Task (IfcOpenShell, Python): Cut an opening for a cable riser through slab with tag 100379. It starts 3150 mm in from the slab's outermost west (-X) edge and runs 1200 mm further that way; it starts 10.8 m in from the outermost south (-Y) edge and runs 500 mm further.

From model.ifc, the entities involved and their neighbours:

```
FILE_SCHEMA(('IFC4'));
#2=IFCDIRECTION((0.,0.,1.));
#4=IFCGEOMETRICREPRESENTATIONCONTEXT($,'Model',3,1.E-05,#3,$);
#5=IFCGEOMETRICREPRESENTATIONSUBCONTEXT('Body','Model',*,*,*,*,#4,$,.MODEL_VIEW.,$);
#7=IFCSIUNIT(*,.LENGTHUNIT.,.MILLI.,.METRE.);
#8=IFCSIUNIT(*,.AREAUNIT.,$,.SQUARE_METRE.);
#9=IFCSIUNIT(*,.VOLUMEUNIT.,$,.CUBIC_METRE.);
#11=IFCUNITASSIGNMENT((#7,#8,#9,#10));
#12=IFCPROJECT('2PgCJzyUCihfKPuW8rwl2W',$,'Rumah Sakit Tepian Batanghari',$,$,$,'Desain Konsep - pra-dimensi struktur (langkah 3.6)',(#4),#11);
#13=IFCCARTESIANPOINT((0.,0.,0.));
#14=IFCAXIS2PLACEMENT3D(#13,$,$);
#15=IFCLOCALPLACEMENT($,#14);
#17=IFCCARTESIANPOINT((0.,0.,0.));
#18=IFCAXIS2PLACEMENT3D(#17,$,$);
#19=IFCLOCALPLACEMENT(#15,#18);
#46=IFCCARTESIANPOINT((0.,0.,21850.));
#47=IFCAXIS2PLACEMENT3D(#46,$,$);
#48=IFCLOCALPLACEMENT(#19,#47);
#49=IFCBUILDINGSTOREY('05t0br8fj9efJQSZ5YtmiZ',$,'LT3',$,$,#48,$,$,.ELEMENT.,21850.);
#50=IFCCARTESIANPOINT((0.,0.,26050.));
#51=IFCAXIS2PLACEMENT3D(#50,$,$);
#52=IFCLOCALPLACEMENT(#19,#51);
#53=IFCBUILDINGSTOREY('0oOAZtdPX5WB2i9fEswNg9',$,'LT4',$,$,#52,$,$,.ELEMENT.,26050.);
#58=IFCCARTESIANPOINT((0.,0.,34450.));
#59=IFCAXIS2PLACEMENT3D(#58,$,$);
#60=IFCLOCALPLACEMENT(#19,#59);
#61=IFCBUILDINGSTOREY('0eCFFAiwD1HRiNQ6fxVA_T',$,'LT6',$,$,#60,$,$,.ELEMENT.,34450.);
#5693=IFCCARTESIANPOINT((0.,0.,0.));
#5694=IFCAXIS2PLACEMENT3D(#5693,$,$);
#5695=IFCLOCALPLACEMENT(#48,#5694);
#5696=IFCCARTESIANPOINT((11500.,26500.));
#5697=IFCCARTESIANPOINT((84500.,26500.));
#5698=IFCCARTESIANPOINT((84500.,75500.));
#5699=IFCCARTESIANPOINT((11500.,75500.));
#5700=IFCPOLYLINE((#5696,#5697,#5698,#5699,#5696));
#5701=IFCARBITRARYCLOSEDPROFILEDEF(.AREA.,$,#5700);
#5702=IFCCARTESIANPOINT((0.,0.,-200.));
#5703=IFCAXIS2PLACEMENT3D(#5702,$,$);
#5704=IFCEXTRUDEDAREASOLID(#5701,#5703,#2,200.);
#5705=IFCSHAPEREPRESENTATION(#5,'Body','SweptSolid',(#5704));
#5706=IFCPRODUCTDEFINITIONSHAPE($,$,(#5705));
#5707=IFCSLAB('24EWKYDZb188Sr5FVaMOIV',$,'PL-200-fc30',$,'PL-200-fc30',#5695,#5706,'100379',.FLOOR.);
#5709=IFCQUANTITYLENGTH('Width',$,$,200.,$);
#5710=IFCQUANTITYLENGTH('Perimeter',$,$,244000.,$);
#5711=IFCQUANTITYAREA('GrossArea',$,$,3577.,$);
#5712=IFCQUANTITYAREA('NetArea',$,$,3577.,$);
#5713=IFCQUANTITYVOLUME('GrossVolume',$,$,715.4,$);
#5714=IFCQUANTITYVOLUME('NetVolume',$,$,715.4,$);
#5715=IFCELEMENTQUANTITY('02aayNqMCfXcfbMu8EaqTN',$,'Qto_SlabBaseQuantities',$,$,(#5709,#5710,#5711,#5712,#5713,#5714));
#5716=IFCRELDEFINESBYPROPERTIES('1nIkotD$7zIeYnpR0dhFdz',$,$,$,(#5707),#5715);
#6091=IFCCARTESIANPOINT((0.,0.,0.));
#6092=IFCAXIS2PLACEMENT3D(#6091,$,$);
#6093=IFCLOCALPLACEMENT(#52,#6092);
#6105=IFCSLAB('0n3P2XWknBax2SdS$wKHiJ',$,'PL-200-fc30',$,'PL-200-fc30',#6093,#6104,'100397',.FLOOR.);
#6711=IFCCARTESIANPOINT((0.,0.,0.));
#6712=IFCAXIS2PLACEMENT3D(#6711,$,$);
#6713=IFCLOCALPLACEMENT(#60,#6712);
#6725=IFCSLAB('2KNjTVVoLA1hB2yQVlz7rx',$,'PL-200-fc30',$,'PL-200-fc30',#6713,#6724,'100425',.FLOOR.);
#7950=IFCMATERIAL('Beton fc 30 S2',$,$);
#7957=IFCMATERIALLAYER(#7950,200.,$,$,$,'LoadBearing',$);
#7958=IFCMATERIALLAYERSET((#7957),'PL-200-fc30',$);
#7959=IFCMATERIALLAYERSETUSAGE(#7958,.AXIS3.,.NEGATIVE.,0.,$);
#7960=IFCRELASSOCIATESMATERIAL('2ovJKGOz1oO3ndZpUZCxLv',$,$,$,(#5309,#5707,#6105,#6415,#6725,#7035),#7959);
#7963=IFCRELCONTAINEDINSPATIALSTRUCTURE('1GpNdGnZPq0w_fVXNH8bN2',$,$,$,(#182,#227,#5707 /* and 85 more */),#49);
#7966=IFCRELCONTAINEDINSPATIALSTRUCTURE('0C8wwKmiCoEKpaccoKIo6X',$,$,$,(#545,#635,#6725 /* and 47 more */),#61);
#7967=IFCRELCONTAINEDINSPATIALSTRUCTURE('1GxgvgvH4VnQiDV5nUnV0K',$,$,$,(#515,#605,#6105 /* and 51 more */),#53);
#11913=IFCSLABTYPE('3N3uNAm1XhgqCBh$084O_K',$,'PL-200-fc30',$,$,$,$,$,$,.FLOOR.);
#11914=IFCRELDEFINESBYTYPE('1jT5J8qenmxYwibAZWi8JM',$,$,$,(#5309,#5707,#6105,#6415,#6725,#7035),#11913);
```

```python
import numpy as np
import ifcopenshell
import ifcopenshell.api.feature
import ifcopenshell.api.geometry
import ifcopenshell.api.pset
import ifcopenshell.api.root
import ifcopenshell.geom
import ifcopenshell.util.element
import ifcopenshell.util.placement
import ifcopenshell.util.representation
import ifcopenshell.util.shape
import ifcopenshell.util.unit

model = ifcopenshell.open("model.ifc")
unit_scale = ifcopenshell.util.unit.calculate_unit_scale(model)
area_scale = ifcopenshell.util.unit.calculate_unit_scale(model, "AREAUNIT")
volume_scale = ifcopenshell.util.unit.calculate_unit_scale(model, "VOLUMEUNIT")
settings = ifcopenshell.geom.settings()


def volume(element):
    """Net volume in cubic metres, openings subtracted."""
    shape = ifcopenshell.geom.create_shape(settings, element)
    return ifcopenshell.util.shape.get_volume(shape.geometry)


slab = model.by_id(5707)
before = volume(slab)

# Extent in the slab's own axes, in metres. The edges named are its -X and -Y sides.
slab_shape = ifcopenshell.geom.create_shape(settings, slab)
vertices = ifcopenshell.util.shape.get_vertices(slab_shape.geometry)
x_min, y_min, bottom = vertices.min(axis=0)
top = vertices[:, 2].max()

opening = ifcopenshell.api.root.create_entity(model, ifc_class="IfcOpeningElement", name="Cable riser opening", predefined_type="OPENING")
context = ifcopenshell.util.representation.get_context(model, "Model", "Body", "MODEL_VIEW")
width, depth = 1.2, 0.5
outline = [(0.0, 0.0), (width, 0.0), (width, depth), (0.0, depth), (0.0, 0.0)]
# Overshoot both faces by 50 mm so the cut is clean.
shape = ifcopenshell.api.geometry.add_slab_representation(
    model, context=context, depth=top - bottom + 0.1, polyline=outline
)
ifcopenshell.api.geometry.assign_representation(model, product=opening, representation=shape)

matrix = ifcopenshell.util.placement.get_local_placement(slab.ObjectPlacement)
matrix[:, 3] = matrix @ np.append(np.array([x_min + 3.15, y_min + 10.8, bottom - 0.05]) / unit_scale, 1.0)
ifcopenshell.api.geometry.edit_object_placement(model, product=opening, matrix=matrix, is_si=False)
ifcopenshell.api.feature.add_feature(model, feature=opening, element=slab)

after = volume(slab)

# Update the slab's stored quantities.
qto = model.by_id(ifcopenshell.util.element.get_pset(slab, "Qto_SlabBaseQuantities", should_inherit=False)["id"])
ifcopenshell.api.pset.edit_qto(model, qto=qto, properties={
    "NetArea": after / (top - bottom) / area_scale,
    "NetVolume": after / volume_scale,
})

print(f"slab volume {before:.3f} -> {after:.3f} m3")

model.write("model_updated.ifc")
```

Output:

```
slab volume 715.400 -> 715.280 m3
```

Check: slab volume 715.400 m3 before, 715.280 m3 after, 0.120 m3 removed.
